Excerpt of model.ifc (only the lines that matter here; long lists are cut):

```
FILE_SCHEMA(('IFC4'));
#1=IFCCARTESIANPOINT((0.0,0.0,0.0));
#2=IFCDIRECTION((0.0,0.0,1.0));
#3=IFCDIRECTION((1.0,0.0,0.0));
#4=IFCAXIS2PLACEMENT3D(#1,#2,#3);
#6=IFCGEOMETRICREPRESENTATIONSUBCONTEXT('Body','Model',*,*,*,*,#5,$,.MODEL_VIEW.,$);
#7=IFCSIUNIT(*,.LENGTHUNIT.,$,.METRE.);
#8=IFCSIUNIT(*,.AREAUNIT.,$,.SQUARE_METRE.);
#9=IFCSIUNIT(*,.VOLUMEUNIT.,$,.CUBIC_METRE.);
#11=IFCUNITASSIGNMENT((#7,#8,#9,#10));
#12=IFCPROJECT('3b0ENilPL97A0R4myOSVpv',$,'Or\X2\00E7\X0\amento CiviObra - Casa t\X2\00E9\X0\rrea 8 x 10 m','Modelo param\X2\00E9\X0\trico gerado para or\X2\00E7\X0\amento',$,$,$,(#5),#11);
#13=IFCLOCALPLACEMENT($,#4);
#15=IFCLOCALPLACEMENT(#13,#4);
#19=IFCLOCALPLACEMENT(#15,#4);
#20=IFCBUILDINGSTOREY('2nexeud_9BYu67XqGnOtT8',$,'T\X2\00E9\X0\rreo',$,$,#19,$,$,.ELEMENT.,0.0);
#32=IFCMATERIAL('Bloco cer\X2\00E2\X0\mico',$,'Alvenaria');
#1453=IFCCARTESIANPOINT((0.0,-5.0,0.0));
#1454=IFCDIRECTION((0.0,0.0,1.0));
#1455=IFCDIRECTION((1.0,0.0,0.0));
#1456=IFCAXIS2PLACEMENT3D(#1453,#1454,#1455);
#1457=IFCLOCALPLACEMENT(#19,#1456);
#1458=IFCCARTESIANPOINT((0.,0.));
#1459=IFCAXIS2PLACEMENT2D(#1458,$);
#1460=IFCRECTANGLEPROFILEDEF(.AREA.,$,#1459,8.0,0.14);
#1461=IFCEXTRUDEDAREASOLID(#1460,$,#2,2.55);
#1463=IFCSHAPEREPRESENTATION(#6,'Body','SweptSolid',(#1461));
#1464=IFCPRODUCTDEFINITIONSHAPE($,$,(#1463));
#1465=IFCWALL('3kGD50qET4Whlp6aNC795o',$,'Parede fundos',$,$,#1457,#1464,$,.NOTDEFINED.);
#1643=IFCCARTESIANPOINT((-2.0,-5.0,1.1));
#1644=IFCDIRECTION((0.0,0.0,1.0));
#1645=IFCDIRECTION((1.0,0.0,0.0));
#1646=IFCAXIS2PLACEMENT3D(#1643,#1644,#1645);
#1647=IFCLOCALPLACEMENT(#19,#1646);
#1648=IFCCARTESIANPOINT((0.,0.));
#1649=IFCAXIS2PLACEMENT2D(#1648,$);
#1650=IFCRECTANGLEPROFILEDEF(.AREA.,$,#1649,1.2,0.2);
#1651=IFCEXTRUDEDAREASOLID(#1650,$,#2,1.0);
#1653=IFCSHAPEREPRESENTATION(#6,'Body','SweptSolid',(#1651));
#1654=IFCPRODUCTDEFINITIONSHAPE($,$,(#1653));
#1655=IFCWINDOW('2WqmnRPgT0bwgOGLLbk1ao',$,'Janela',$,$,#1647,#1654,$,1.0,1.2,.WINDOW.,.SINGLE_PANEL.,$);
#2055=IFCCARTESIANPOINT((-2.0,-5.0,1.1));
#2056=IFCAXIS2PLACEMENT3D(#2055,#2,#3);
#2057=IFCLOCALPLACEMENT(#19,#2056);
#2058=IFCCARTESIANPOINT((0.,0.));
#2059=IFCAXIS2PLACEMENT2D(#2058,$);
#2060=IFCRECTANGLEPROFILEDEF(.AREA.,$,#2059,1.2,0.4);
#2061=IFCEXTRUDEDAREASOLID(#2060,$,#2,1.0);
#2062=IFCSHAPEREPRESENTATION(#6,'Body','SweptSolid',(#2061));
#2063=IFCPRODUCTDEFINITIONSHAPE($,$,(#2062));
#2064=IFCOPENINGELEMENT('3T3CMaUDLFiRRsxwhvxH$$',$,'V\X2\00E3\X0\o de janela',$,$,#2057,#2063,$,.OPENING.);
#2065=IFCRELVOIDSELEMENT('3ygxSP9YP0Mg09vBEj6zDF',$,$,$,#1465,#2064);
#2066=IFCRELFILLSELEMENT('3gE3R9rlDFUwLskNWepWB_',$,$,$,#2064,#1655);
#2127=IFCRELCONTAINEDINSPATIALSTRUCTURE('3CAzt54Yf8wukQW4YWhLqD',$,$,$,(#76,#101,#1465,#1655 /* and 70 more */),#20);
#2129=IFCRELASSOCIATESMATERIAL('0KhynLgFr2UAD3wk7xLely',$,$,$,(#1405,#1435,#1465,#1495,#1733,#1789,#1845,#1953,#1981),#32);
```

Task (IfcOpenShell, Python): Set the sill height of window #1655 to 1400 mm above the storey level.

```python
import numpy as np
import ifcopenshell
import ifcopenshell.api.geometry
import ifcopenshell.geom
import ifcopenshell.util.element
import ifcopenshell.util.placement
import ifcopenshell.util.shape
import ifcopenshell.util.unit

model = ifcopenshell.open("model.ifc")
unit_scale = ifcopenshell.util.unit.calculate_unit_scale(model)

window = model.by_guid("2WqmnRPgT0bwgOGLLbk1ao")
opening = window.FillsVoids[0].RelatingOpeningElement
storey = ifcopenshell.util.element.get_container(window, ifc_class="IfcBuildingStorey")
level = ifcopenshell.util.placement.get_local_placement(storey.ObjectPlacement)[2, 3]

# The opening's origin need not be at the sill, so measure its lowest point.
shape = ifcopenshell.geom.create_shape(ifcopenshell.geom.settings(), opening)
bottom = ifcopenshell.util.shape.get_shape_bottom_elevation(shape, shape.geometry) / unit_scale
dz = level + 1.4 / unit_scale - bottom

shift = np.array([0.0, 0.0, dz])
# The window is not placed relative to its opening, so move both.
for product in (opening, window):
    matrix = ifcopenshell.util.placement.get_local_placement(product.ObjectPlacement)
    matrix[:3, 3] += shift
    ifcopenshell.api.geometry.edit_object_placement(model, product=product, matrix=matrix, is_si=False)

print(f"moved by {dz * unit_scale:+.3f} m")

model.write("model_updated.ifc")
```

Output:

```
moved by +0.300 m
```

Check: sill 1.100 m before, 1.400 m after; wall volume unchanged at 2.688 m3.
